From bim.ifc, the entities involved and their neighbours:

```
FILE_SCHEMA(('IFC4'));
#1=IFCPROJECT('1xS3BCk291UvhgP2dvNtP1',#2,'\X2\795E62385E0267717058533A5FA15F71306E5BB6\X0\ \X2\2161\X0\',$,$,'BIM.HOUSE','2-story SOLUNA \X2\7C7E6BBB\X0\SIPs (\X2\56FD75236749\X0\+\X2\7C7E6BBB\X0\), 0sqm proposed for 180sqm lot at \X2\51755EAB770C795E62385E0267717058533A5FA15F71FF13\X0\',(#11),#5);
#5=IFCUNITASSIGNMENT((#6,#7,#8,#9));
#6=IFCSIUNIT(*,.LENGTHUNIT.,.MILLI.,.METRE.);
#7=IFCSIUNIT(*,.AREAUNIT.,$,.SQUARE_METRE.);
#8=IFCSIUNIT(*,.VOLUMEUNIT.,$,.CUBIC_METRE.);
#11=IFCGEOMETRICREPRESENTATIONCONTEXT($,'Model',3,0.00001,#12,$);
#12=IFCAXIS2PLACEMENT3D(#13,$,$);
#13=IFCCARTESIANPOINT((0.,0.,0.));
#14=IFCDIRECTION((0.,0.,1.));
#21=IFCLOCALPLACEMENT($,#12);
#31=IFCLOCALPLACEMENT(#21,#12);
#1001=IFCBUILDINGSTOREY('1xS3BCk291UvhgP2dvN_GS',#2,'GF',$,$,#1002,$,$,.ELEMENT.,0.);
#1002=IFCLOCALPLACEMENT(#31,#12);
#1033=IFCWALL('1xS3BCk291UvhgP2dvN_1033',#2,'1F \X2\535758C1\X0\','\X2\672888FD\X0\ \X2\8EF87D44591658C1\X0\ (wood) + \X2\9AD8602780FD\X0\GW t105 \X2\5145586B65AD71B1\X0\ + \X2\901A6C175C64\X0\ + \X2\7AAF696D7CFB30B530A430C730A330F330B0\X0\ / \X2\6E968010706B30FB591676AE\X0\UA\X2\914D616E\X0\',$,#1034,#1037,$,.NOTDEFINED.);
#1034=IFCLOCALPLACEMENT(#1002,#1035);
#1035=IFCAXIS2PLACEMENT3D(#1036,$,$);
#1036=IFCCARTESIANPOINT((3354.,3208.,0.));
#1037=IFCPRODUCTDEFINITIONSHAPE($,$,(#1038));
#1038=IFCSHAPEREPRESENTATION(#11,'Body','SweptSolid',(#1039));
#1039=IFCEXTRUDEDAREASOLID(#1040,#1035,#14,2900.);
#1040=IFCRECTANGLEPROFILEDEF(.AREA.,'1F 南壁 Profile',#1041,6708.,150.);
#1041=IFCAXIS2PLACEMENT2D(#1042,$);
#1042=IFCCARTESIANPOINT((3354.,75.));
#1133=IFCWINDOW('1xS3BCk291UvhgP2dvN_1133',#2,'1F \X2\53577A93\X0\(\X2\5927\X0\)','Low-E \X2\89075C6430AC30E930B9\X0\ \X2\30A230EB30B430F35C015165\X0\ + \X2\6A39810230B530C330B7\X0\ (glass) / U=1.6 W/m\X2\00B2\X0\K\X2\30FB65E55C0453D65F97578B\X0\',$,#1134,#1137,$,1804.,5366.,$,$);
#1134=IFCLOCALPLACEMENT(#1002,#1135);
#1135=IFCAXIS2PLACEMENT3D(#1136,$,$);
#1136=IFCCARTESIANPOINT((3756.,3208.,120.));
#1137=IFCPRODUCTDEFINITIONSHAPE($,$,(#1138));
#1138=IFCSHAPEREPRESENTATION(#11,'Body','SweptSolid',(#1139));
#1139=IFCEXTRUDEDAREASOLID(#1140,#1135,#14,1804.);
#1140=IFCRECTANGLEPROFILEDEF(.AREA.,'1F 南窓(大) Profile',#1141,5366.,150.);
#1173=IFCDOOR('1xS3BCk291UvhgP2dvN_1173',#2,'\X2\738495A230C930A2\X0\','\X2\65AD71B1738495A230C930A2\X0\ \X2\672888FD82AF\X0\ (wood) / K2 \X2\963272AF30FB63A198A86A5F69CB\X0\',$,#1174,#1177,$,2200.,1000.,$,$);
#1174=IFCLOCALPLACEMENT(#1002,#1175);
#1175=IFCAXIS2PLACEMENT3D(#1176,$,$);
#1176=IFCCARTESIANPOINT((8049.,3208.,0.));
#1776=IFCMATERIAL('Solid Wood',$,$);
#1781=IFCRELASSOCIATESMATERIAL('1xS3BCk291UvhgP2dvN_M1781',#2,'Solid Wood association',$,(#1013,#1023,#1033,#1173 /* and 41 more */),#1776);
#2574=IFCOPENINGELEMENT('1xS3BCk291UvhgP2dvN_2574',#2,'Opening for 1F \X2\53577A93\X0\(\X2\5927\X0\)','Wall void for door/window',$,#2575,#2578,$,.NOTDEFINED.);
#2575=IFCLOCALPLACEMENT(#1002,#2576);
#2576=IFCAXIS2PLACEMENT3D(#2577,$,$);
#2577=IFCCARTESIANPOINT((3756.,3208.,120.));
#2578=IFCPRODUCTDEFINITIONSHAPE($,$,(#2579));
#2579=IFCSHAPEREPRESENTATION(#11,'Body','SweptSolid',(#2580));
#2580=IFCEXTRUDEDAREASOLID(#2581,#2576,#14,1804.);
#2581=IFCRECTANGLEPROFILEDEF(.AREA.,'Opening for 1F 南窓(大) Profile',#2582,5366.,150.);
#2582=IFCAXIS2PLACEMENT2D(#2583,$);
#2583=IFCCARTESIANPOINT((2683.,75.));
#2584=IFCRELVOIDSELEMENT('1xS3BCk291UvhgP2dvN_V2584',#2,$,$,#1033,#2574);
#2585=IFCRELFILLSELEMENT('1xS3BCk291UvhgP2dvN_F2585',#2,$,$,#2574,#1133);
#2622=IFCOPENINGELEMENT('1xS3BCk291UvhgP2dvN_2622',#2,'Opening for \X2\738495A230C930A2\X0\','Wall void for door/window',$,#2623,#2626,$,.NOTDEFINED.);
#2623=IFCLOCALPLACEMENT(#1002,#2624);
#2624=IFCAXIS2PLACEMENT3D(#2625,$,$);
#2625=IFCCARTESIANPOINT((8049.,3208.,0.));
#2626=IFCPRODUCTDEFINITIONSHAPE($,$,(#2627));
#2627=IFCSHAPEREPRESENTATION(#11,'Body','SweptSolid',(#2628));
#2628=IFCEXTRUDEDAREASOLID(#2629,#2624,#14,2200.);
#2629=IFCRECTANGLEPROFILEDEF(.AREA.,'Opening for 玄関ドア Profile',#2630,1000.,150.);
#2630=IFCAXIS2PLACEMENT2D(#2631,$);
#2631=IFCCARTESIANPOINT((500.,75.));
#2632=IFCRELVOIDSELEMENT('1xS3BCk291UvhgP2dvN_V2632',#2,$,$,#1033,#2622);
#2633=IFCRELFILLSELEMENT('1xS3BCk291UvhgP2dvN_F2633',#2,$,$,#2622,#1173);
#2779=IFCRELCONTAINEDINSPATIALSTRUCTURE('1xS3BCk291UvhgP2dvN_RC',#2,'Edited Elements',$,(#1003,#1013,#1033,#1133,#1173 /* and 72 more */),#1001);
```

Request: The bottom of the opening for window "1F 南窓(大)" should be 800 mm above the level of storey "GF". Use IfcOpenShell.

```python
import numpy as np
import ifcopenshell
import ifcopenshell.api.geometry
import ifcopenshell.geom
import ifcopenshell.util.element
import ifcopenshell.util.placement
import ifcopenshell.util.shape
import ifcopenshell.util.unit

model = ifcopenshell.open("bim.ifc")
unit_scale = ifcopenshell.util.unit.calculate_unit_scale(model)

window = model.by_id(1133)
opening = window.FillsVoids[0].RelatingOpeningElement
storey = ifcopenshell.util.element.get_container(window, ifc_class="IfcBuildingStorey")
level = ifcopenshell.util.placement.get_local_placement(storey.ObjectPlacement)[2, 3]

# The opening's origin need not be at the sill, so measure its lowest point.
shape = ifcopenshell.geom.create_shape(ifcopenshell.geom.settings(), opening)
bottom = ifcopenshell.util.shape.get_shape_bottom_elevation(shape, shape.geometry) / unit_scale
dz = level + 0.8 / unit_scale - bottom

shift = np.array([0.0, 0.0, dz])
# The window is not placed relative to its opening, so move both.
for product in (opening, window):
    matrix = ifcopenshell.util.placement.get_local_placement(product.ObjectPlacement)
    matrix[:3, 3] += shift
    ifcopenshell.api.geometry.edit_object_placement(model, product=product, matrix=matrix, is_si=False)

print(f"moved by {dz * unit_scale:+.3f} m")

model.write("bim_edited.ifc")
```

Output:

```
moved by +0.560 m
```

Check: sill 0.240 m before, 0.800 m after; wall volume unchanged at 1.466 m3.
